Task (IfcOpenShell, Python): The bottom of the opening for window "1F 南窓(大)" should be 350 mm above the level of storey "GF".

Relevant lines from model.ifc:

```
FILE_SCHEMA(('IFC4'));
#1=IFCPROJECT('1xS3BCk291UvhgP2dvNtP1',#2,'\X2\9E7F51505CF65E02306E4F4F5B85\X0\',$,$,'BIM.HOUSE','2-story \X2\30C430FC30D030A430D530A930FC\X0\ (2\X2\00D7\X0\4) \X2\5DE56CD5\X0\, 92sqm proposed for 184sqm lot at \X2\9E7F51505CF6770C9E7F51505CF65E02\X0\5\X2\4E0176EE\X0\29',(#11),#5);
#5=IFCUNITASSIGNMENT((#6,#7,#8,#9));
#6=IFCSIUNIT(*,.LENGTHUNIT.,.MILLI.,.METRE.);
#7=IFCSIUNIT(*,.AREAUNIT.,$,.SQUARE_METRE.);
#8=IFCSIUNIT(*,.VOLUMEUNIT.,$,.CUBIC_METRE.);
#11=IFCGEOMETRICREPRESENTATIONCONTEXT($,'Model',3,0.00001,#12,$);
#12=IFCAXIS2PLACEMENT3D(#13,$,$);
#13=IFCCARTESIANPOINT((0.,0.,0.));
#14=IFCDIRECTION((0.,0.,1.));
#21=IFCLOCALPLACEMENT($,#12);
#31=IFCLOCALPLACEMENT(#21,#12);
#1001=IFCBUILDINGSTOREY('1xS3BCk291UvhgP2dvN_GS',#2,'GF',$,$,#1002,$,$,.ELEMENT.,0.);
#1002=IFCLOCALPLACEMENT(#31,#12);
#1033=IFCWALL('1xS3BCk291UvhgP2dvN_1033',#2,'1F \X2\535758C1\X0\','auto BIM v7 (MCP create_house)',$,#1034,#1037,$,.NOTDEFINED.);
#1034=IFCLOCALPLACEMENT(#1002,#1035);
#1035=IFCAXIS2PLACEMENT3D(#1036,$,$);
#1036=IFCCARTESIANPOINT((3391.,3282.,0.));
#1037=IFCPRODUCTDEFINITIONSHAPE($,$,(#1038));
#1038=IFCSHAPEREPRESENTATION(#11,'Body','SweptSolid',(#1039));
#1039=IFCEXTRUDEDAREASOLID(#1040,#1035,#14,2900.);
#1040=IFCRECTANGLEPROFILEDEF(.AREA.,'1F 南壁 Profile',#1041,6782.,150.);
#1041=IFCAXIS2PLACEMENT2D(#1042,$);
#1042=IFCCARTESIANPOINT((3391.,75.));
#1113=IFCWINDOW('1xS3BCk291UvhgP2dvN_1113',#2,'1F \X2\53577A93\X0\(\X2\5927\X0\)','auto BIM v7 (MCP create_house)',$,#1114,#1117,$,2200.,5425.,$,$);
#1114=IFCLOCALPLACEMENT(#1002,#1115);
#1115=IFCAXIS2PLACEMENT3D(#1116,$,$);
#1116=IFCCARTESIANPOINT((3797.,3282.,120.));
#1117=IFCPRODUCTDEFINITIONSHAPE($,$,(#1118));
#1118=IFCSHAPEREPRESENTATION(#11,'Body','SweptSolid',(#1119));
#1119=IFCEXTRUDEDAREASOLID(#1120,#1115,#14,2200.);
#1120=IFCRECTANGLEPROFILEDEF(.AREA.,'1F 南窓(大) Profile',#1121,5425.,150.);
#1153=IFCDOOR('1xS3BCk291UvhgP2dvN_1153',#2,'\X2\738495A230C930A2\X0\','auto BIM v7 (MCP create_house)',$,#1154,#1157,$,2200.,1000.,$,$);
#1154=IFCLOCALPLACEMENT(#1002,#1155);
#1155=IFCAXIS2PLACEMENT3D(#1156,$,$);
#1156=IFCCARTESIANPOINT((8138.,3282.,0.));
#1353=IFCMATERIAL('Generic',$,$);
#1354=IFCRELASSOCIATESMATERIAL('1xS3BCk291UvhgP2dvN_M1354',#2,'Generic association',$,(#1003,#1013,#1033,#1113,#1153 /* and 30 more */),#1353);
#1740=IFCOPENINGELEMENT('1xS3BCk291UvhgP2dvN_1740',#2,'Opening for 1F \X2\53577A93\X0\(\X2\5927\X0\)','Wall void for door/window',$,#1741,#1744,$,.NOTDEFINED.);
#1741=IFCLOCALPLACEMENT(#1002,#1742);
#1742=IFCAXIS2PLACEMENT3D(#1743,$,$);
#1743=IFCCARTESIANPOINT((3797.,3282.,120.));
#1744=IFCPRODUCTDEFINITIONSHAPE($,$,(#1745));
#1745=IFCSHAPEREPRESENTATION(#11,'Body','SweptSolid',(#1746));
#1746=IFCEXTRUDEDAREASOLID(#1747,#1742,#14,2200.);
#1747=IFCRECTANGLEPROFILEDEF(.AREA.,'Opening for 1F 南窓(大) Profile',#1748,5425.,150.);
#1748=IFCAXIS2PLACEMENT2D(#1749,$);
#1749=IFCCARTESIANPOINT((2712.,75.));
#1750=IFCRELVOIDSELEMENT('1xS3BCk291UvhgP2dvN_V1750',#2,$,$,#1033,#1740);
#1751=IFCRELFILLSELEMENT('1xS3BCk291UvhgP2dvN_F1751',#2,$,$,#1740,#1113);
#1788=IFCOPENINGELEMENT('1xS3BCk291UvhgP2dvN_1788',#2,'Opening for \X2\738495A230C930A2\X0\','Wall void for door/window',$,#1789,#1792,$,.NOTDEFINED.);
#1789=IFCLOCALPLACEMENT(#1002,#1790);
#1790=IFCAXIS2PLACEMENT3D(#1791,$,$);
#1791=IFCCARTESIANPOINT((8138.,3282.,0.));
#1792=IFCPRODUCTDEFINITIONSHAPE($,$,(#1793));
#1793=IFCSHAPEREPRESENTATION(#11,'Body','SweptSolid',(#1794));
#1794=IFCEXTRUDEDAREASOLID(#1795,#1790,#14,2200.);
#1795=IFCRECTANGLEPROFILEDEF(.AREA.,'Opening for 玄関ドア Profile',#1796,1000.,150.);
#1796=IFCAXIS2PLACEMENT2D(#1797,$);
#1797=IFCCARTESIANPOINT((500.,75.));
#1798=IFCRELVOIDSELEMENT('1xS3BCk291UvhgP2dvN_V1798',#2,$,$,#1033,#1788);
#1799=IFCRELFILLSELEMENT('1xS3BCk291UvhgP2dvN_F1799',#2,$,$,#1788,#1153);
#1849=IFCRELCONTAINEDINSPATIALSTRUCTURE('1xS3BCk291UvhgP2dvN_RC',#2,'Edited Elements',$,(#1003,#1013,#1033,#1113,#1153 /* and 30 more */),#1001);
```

```python
import numpy as np
import ifcopenshell
import ifcopenshell.api.geometry
import ifcopenshell.geom
import ifcopenshell.util.element
import ifcopenshell.util.placement
import ifcopenshell.util.shape
import ifcopenshell.util.unit

model = ifcopenshell.open("model.ifc")
unit_scale = ifcopenshell.util.unit.calculate_unit_scale(model)

window = model.by_guid("1xS3BCk291UvhgP2dvN_1113")
opening = window.FillsVoids[0].RelatingOpeningElement
storey = ifcopenshell.util.element.get_container(window, ifc_class="IfcBuildingStorey")
level = ifcopenshell.util.placement.get_local_placement(storey.ObjectPlacement)[2, 3]

# The opening's origin need not be at the sill, so measure its lowest point.
shape = ifcopenshell.geom.create_shape(ifcopenshell.geom.settings(), opening)
bottom = ifcopenshell.util.shape.get_shape_bottom_elevation(shape, shape.geometry) / unit_scale
dz = level + 0.35 / unit_scale - bottom

shift = np.array([0.0, 0.0, dz])
# The window is not placed relative to its opening, so move both.
for product in (opening, window):
    matrix = ifcopenshell.util.placement.get_local_placement(product.ObjectPlacement)
    matrix[:3, 3] += shift
    ifcopenshell.api.geometry.edit_object_placement(model, product=product, matrix=matrix, is_si=False)

print(f"moved by {dz * unit_scale:+.3f} m")

model.write("model_rev.ifc")
```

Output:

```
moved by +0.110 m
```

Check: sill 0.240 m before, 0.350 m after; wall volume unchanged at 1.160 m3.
